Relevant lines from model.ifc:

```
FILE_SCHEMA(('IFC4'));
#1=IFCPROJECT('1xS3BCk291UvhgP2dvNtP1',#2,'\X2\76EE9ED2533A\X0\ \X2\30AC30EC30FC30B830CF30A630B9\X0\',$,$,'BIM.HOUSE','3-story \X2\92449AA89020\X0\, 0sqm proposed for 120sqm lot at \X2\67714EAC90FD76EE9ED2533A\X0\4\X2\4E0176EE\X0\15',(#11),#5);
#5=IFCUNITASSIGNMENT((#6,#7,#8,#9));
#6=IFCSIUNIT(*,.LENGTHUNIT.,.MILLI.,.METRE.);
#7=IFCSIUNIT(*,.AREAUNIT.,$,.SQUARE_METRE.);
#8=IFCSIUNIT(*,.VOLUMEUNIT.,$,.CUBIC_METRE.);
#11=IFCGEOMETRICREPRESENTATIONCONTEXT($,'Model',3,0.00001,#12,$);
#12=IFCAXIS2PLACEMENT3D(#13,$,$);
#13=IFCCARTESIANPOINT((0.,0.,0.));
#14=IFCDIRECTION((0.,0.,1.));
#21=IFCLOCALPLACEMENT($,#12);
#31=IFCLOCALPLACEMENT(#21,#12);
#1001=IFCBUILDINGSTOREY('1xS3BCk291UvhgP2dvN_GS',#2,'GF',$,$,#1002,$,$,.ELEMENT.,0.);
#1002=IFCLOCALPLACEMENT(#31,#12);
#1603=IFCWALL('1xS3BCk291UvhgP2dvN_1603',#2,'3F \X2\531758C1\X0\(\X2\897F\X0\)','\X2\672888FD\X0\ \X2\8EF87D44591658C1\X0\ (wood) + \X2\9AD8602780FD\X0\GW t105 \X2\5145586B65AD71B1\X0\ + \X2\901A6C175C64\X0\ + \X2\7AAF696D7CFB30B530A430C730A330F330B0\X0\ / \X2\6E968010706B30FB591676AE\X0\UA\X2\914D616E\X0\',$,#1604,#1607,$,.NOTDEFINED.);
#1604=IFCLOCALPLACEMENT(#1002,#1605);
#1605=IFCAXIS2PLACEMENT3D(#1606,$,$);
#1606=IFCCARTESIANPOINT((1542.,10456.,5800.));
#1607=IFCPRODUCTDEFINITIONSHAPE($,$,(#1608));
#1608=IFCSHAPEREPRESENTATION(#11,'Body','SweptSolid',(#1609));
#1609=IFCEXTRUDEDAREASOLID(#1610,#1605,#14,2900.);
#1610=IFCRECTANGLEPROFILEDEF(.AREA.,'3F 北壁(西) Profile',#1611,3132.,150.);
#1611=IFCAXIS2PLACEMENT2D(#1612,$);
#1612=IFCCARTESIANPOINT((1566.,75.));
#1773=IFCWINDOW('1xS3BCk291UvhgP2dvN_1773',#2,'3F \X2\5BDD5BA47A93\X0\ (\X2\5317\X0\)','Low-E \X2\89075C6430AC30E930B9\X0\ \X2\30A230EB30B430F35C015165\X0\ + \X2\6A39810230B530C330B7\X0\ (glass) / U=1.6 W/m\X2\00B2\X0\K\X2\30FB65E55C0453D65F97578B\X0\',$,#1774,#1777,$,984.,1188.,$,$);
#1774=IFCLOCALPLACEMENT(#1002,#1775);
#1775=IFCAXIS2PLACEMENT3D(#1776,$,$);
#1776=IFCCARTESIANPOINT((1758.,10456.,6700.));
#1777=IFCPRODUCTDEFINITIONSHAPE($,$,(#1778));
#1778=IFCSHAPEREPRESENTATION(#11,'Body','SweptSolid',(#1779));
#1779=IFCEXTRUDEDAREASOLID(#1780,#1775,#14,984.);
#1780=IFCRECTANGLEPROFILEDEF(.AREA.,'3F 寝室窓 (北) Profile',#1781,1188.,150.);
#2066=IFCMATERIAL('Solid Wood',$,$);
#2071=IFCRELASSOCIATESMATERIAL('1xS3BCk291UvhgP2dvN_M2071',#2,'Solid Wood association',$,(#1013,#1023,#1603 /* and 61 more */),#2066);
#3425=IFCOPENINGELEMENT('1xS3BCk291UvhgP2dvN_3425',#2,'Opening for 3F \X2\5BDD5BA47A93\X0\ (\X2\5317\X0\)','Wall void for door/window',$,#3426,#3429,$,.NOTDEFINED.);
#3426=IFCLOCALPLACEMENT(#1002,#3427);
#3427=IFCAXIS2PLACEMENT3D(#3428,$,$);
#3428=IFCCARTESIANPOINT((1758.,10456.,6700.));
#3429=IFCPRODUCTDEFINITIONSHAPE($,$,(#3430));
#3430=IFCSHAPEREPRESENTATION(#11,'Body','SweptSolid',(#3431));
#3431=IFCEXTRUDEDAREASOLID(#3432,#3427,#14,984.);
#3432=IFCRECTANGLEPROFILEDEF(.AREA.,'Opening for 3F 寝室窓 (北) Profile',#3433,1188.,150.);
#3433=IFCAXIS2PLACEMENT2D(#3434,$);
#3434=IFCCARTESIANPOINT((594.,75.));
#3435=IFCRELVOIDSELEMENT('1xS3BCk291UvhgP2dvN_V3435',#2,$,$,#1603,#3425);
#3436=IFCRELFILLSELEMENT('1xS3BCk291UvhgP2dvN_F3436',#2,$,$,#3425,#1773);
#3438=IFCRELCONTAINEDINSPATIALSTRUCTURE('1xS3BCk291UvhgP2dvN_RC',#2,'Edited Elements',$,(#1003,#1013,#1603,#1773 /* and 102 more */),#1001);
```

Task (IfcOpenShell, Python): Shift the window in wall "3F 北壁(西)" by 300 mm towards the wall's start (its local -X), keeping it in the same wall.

```python
import ifcopenshell
import ifcopenshell.api.geometry
import ifcopenshell.util.placement

model = ifcopenshell.open("model.ifc")

window = model.by_guid("1xS3BCk291UvhgP2dvN_1773")
opening = window.FillsVoids[0].RelatingOpeningElement
wall = opening.VoidsElements[0].RelatingBuildingElement

wall_matrix = ifcopenshell.util.placement.get_local_placement(wall.ObjectPlacement)
shift = wall_matrix[:3, 0] * -300.0
before = ifcopenshell.util.placement.get_local_placement(window.ObjectPlacement)[:3, 3].copy()

# The window is not placed relative to its opening, so move both.
for product in (opening, window):
    matrix = ifcopenshell.util.placement.get_local_placement(product.ObjectPlacement)
    matrix[:3, 3] += shift
    ifcopenshell.api.geometry.edit_object_placement(model, product=product, matrix=matrix, is_si=False)

after = ifcopenshell.util.placement.get_local_placement(window.ObjectPlacement)[:3, 3]
print("window moved by", (after - before).round(3) + 0.0)

model.write("model_updated.ifc")
```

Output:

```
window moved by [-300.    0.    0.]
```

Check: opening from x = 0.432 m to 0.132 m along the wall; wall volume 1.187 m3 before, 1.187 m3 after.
